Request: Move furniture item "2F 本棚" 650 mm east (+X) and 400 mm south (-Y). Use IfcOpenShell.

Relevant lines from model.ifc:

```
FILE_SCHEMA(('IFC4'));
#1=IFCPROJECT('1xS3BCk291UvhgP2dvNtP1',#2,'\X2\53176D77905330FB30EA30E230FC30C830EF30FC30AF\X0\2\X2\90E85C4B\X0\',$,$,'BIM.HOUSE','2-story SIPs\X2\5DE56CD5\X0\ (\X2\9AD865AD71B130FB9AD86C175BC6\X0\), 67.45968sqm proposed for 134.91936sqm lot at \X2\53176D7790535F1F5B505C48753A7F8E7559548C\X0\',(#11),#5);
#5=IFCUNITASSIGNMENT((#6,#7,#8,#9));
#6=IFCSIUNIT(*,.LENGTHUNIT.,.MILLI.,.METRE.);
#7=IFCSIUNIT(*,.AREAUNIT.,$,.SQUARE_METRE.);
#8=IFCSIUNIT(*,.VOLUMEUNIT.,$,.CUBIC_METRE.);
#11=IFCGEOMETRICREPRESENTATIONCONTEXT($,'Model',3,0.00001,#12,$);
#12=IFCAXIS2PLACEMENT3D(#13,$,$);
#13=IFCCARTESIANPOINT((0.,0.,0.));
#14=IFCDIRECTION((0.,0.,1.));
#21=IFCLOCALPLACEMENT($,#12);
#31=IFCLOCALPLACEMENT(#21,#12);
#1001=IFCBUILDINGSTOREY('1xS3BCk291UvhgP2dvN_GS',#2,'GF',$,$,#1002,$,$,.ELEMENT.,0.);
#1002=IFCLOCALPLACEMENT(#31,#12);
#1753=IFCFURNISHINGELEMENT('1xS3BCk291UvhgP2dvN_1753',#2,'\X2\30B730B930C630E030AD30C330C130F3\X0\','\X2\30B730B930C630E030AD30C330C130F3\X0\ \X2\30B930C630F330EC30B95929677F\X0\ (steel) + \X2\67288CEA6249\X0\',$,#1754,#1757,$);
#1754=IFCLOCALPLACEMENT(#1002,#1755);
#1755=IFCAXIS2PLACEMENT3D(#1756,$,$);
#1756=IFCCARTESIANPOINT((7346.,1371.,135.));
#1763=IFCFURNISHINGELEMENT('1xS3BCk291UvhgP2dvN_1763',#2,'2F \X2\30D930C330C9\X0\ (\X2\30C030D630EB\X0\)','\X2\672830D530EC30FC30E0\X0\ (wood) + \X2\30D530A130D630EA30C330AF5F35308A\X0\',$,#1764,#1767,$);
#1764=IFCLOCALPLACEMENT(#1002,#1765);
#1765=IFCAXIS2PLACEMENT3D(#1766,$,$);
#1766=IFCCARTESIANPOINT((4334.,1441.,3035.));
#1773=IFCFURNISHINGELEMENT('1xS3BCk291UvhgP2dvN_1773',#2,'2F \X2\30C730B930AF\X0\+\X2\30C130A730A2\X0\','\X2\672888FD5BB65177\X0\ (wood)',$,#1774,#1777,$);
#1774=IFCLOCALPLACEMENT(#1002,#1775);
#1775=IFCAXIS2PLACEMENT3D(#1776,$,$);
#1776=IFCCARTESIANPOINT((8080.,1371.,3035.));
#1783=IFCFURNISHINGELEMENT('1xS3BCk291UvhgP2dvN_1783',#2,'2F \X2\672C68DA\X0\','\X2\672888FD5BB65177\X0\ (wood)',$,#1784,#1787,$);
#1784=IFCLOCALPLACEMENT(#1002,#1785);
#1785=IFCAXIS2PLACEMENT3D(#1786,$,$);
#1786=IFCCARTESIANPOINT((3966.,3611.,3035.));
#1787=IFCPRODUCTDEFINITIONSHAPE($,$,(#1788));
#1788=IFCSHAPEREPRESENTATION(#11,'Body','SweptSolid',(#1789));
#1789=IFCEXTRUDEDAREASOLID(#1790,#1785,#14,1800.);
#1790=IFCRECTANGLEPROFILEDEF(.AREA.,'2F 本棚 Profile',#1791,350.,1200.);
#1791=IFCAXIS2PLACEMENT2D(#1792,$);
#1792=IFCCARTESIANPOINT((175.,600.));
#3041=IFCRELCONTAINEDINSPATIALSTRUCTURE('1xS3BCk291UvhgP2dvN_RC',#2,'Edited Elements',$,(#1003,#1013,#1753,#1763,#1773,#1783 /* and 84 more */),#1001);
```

```python
import ifcopenshell
import ifcopenshell.api.geometry
import ifcopenshell.util.placement

model = ifcopenshell.open("model.ifc")

item = model.by_guid("1xS3BCk291UvhgP2dvN_1783")
matrix = ifcopenshell.util.placement.get_local_placement(item.ObjectPlacement)
matrix[0, 3] += 650.0
matrix[1, 3] -= 400.0
ifcopenshell.api.geometry.edit_object_placement(model, product=item, matrix=matrix, is_si=False)

print(ifcopenshell.util.placement.get_local_placement(item.ObjectPlacement).round(3) + 0.0)

model.write("model_rev.ifc")
```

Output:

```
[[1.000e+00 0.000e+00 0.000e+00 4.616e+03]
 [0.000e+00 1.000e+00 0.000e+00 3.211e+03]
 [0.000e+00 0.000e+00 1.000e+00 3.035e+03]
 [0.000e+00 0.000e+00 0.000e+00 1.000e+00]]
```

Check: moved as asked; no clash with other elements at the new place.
